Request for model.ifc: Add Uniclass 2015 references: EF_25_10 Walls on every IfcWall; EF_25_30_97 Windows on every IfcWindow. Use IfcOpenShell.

First a look at what the model holds.

```python
import ifcopenshell

model = ifcopenshell.open("model.ifc")
print(model.schema)
print("classifications:", [c.Name for c in model.by_type("IfcClassification")])
for ifc_class in ("IfcDoor", "IfcRoof", "IfcStair", "IfcWall", "IfcWindow"):
    print(ifc_class, len(model.by_type(ifc_class)))
```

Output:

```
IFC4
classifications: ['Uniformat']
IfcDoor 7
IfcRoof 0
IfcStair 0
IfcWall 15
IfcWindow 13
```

```python
import ifcopenshell
import ifcopenshell.api.classification

model = ifcopenshell.open("model.ifc")

system = ifcopenshell.api.classification.add_classification(model, classification="Uniclass 2015")

codes = {
    "IfcWall": ("EF_25_10", "Walls"),
    "IfcWindow": ("EF_25_30_97", "Windows"),
}
for ifc_class, (code, name) in codes.items():
    products = model.by_type(ifc_class)
    ifcopenshell.api.classification.add_reference(
        model, products=products, classification=system, identification=code, name=name
    )
    print(code, len(products))

model.write("model_rev.ifc")
```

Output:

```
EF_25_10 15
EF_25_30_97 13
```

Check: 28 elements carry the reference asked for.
